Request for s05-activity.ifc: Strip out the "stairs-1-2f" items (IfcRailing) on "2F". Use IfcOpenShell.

First a look at what the model holds.

```python
import ifcopenshell
import ifcopenshell.util.element

model = ifcopenshell.open("s05-activity.ifc")
print(model.schema)
storey = next(s for s in model.by_type("IfcBuildingStorey") if s.Name == "2F")
railings = [e for e in ifcopenshell.util.element.get_decomposition(storey) if e.is_a("IfcRailing")]
seen = {}
for e in railings:
    element_type = ifcopenshell.util.element.get_type(e)
    name = element_type.Name if element_type not in (None, e) else None
    seen[name] = seen.get(name, 0) + 1
for name, count in sorted(seen.items(), key=str):
    print(count, "x", name)
```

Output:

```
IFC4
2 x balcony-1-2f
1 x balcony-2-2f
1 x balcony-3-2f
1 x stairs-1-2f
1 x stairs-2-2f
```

```python
import ifcopenshell
import ifcopenshell.api.root
import ifcopenshell.util.element

model = ifcopenshell.open("s05-activity.ifc")

storey = next(s for s in model.by_type("IfcBuildingStorey") if s.Name == "2F")
railings = [e for e in ifcopenshell.util.element.get_decomposition(storey) if e.is_a("IfcRailing")]
targets = [e for e in railings if (t := ifcopenshell.util.element.get_type(e)) not in (None, e) and t.Name == "stairs-1-2f"]

for e in targets:
    ifcopenshell.api.root.remove_product(model, product=e)
print(len(targets), "removed")

model.write("s05-activity_rev.ifc")
```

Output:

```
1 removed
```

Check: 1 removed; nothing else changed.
